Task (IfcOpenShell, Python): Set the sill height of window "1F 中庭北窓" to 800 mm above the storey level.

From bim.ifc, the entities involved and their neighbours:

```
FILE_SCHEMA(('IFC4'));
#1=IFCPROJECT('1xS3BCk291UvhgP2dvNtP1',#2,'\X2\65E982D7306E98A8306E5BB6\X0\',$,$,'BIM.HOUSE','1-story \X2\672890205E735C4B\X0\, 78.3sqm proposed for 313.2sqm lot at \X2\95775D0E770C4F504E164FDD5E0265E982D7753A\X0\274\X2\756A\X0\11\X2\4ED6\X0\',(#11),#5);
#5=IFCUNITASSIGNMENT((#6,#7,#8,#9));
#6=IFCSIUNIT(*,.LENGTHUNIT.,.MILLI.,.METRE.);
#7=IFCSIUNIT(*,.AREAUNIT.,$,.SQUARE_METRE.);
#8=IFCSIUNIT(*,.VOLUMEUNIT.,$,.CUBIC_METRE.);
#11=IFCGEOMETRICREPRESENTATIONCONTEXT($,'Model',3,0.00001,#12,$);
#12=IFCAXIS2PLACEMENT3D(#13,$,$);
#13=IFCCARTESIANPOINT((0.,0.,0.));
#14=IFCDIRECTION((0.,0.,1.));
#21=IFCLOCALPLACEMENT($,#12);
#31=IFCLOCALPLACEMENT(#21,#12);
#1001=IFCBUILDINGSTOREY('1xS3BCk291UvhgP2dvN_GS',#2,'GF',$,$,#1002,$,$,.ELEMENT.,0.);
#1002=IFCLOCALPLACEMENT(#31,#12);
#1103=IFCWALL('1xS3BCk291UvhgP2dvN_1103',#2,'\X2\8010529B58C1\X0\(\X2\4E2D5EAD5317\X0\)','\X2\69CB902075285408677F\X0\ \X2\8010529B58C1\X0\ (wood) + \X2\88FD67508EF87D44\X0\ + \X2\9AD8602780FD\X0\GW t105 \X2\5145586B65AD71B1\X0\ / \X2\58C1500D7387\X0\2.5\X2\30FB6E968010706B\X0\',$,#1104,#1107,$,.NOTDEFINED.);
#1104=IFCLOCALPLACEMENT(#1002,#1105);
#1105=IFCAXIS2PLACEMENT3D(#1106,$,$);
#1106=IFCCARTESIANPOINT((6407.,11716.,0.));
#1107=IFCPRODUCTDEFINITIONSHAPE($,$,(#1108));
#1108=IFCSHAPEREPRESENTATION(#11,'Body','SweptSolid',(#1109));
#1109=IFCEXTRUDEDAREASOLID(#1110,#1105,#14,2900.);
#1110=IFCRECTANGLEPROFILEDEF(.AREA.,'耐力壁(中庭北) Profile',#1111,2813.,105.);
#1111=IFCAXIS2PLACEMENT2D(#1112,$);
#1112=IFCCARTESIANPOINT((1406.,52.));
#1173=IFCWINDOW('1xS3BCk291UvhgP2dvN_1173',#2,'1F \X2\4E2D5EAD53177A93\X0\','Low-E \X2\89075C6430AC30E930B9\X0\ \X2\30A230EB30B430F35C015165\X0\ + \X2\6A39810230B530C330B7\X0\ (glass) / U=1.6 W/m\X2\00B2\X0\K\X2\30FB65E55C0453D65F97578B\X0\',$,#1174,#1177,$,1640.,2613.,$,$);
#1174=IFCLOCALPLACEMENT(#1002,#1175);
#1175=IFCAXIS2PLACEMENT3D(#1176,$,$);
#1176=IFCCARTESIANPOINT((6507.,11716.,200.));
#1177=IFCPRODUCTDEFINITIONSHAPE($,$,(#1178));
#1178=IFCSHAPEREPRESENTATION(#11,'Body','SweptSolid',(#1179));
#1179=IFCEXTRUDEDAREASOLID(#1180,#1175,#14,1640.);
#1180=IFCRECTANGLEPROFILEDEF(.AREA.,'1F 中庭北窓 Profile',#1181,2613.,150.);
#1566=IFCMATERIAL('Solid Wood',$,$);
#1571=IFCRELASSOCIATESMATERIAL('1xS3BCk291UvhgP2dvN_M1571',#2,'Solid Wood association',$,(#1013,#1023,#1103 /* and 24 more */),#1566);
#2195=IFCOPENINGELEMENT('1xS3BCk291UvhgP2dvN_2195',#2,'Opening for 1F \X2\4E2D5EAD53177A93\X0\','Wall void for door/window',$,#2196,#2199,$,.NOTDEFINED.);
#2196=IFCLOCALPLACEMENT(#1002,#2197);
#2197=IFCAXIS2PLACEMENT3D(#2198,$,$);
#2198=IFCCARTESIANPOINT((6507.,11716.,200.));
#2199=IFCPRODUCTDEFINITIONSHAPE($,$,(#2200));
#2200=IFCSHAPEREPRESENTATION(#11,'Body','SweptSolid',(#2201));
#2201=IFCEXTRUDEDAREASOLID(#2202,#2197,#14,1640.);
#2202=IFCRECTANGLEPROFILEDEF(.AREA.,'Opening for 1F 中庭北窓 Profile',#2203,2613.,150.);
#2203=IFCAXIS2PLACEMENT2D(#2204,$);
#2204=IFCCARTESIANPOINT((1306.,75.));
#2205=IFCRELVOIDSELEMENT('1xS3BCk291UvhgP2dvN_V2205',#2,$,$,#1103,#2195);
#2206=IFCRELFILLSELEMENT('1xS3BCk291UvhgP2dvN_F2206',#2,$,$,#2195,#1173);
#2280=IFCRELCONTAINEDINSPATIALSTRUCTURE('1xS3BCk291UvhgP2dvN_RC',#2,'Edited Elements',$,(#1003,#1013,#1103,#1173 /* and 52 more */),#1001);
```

```python
import numpy as np
import ifcopenshell
import ifcopenshell.api.geometry
import ifcopenshell.geom
import ifcopenshell.util.element
import ifcopenshell.util.placement
import ifcopenshell.util.shape
import ifcopenshell.util.unit

model = ifcopenshell.open("bim.ifc")
unit_scale = ifcopenshell.util.unit.calculate_unit_scale(model)

window = model.by_guid("1xS3BCk291UvhgP2dvN_1173")
opening = window.FillsVoids[0].RelatingOpeningElement
storey = ifcopenshell.util.element.get_container(window, ifc_class="IfcBuildingStorey")
level = ifcopenshell.util.placement.get_local_placement(storey.ObjectPlacement)[2, 3]

# The opening's origin need not be at the sill, so measure its lowest point.
shape = ifcopenshell.geom.create_shape(ifcopenshell.geom.settings(), opening)
bottom = ifcopenshell.util.shape.get_shape_bottom_elevation(shape, shape.geometry) / unit_scale
dz = level + 800.0 - bottom

shift = np.array([0.0, 0.0, dz])
# The window is not placed relative to its opening, so move both.
for product in (opening, window):
    matrix = ifcopenshell.util.placement.get_local_placement(product.ObjectPlacement)
    matrix[:3, 3] += shift
    ifcopenshell.api.geometry.edit_object_placement(model, product=product, matrix=matrix, is_si=False)

print(f"moved by {dz * unit_scale:+.3f} m")

model.write("bim-out.ifc")
```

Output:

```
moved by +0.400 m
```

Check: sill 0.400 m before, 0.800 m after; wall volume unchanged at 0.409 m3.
